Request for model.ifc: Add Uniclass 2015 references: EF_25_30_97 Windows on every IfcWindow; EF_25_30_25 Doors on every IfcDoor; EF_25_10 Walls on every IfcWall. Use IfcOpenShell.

First a look at what the model holds.

```python
import ifcopenshell

model = ifcopenshell.open("model.ifc")
print(model.schema)
print("classifications:", [c.Name for c in model.by_type("IfcClassification")])
for ifc_class in ("IfcDoor", "IfcRoof", "IfcStair", "IfcWall", "IfcWindow"):
    print(ifc_class, len(model.by_type(ifc_class)))
```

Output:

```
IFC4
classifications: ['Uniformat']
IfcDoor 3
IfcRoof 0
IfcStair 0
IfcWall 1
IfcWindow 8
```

```python
import ifcopenshell
import ifcopenshell.api.classification

model = ifcopenshell.open("model.ifc")

system = ifcopenshell.api.classification.add_classification(model, classification="Uniclass 2015")

codes = {
    "IfcWindow": ("EF_25_30_97", "Windows"),
    "IfcDoor": ("EF_25_30_25", "Doors"),
    "IfcWall": ("EF_25_10", "Walls"),
}
for ifc_class, (code, name) in codes.items():
    products = model.by_type(ifc_class)
    ifcopenshell.api.classification.add_reference(
        model, products=products, classification=system, identification=code, name=name
    )
    print(code, len(products))

model.write("model-out.ifc")
```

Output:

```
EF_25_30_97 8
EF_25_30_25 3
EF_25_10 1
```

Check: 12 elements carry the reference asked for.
